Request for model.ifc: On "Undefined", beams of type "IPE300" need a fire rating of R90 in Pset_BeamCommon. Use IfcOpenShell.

First a look at what the model holds.

```python
import ifcopenshell
import ifcopenshell.util.element

model = ifcopenshell.open("model.ifc")
print(model.schema)
storey = next(s for s in model.by_type("IfcBuildingStorey") if s.Name == "Undefined")
beams = [e for e in ifcopenshell.util.element.get_decomposition(storey) if e.is_a("IfcBeam")]
seen = {}
for e in beams:
    element_type = ifcopenshell.util.element.get_type(e)
    key = (element_type.Name if element_type != e and element_type else None, ifcopenshell.util.element.get_pset(e, "Pset_BeamCommon", "FireRating"))
    seen[key] = seen.get(key, 0) + 1
for (name, value), count in sorted(seen.items(), key=str):
    print(count, "x", name, "|", value)
```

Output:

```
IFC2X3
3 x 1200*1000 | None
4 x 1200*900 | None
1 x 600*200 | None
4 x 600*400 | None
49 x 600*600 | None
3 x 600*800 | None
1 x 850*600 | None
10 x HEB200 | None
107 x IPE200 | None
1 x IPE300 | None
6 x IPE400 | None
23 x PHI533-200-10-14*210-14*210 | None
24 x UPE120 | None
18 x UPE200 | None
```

```python
import ifcopenshell
import ifcopenshell.api.pset
import ifcopenshell.util.element

model = ifcopenshell.open("model.ifc")

storey = next(s for s in model.by_type("IfcBuildingStorey") if s.Name == "Undefined")
beams = [e for e in ifcopenshell.util.element.get_decomposition(storey) if e.is_a("IfcBeam")]

count = 0
for e in beams:
    element_type = ifcopenshell.util.element.get_type(e)
    if element_type in (None, e) or element_type.Name != "IPE300":
        continue
    # add_pset returns the element's existing set when there is one.
    pset = ifcopenshell.api.pset.add_pset(model, product=e, name="Pset_BeamCommon")
    ifcopenshell.api.pset.edit_pset(model, pset=pset, properties={"FireRating": "R90"})
    count += 1

print(count, "beams updated")

model.write("model_rev.ifc")
```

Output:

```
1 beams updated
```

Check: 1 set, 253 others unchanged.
